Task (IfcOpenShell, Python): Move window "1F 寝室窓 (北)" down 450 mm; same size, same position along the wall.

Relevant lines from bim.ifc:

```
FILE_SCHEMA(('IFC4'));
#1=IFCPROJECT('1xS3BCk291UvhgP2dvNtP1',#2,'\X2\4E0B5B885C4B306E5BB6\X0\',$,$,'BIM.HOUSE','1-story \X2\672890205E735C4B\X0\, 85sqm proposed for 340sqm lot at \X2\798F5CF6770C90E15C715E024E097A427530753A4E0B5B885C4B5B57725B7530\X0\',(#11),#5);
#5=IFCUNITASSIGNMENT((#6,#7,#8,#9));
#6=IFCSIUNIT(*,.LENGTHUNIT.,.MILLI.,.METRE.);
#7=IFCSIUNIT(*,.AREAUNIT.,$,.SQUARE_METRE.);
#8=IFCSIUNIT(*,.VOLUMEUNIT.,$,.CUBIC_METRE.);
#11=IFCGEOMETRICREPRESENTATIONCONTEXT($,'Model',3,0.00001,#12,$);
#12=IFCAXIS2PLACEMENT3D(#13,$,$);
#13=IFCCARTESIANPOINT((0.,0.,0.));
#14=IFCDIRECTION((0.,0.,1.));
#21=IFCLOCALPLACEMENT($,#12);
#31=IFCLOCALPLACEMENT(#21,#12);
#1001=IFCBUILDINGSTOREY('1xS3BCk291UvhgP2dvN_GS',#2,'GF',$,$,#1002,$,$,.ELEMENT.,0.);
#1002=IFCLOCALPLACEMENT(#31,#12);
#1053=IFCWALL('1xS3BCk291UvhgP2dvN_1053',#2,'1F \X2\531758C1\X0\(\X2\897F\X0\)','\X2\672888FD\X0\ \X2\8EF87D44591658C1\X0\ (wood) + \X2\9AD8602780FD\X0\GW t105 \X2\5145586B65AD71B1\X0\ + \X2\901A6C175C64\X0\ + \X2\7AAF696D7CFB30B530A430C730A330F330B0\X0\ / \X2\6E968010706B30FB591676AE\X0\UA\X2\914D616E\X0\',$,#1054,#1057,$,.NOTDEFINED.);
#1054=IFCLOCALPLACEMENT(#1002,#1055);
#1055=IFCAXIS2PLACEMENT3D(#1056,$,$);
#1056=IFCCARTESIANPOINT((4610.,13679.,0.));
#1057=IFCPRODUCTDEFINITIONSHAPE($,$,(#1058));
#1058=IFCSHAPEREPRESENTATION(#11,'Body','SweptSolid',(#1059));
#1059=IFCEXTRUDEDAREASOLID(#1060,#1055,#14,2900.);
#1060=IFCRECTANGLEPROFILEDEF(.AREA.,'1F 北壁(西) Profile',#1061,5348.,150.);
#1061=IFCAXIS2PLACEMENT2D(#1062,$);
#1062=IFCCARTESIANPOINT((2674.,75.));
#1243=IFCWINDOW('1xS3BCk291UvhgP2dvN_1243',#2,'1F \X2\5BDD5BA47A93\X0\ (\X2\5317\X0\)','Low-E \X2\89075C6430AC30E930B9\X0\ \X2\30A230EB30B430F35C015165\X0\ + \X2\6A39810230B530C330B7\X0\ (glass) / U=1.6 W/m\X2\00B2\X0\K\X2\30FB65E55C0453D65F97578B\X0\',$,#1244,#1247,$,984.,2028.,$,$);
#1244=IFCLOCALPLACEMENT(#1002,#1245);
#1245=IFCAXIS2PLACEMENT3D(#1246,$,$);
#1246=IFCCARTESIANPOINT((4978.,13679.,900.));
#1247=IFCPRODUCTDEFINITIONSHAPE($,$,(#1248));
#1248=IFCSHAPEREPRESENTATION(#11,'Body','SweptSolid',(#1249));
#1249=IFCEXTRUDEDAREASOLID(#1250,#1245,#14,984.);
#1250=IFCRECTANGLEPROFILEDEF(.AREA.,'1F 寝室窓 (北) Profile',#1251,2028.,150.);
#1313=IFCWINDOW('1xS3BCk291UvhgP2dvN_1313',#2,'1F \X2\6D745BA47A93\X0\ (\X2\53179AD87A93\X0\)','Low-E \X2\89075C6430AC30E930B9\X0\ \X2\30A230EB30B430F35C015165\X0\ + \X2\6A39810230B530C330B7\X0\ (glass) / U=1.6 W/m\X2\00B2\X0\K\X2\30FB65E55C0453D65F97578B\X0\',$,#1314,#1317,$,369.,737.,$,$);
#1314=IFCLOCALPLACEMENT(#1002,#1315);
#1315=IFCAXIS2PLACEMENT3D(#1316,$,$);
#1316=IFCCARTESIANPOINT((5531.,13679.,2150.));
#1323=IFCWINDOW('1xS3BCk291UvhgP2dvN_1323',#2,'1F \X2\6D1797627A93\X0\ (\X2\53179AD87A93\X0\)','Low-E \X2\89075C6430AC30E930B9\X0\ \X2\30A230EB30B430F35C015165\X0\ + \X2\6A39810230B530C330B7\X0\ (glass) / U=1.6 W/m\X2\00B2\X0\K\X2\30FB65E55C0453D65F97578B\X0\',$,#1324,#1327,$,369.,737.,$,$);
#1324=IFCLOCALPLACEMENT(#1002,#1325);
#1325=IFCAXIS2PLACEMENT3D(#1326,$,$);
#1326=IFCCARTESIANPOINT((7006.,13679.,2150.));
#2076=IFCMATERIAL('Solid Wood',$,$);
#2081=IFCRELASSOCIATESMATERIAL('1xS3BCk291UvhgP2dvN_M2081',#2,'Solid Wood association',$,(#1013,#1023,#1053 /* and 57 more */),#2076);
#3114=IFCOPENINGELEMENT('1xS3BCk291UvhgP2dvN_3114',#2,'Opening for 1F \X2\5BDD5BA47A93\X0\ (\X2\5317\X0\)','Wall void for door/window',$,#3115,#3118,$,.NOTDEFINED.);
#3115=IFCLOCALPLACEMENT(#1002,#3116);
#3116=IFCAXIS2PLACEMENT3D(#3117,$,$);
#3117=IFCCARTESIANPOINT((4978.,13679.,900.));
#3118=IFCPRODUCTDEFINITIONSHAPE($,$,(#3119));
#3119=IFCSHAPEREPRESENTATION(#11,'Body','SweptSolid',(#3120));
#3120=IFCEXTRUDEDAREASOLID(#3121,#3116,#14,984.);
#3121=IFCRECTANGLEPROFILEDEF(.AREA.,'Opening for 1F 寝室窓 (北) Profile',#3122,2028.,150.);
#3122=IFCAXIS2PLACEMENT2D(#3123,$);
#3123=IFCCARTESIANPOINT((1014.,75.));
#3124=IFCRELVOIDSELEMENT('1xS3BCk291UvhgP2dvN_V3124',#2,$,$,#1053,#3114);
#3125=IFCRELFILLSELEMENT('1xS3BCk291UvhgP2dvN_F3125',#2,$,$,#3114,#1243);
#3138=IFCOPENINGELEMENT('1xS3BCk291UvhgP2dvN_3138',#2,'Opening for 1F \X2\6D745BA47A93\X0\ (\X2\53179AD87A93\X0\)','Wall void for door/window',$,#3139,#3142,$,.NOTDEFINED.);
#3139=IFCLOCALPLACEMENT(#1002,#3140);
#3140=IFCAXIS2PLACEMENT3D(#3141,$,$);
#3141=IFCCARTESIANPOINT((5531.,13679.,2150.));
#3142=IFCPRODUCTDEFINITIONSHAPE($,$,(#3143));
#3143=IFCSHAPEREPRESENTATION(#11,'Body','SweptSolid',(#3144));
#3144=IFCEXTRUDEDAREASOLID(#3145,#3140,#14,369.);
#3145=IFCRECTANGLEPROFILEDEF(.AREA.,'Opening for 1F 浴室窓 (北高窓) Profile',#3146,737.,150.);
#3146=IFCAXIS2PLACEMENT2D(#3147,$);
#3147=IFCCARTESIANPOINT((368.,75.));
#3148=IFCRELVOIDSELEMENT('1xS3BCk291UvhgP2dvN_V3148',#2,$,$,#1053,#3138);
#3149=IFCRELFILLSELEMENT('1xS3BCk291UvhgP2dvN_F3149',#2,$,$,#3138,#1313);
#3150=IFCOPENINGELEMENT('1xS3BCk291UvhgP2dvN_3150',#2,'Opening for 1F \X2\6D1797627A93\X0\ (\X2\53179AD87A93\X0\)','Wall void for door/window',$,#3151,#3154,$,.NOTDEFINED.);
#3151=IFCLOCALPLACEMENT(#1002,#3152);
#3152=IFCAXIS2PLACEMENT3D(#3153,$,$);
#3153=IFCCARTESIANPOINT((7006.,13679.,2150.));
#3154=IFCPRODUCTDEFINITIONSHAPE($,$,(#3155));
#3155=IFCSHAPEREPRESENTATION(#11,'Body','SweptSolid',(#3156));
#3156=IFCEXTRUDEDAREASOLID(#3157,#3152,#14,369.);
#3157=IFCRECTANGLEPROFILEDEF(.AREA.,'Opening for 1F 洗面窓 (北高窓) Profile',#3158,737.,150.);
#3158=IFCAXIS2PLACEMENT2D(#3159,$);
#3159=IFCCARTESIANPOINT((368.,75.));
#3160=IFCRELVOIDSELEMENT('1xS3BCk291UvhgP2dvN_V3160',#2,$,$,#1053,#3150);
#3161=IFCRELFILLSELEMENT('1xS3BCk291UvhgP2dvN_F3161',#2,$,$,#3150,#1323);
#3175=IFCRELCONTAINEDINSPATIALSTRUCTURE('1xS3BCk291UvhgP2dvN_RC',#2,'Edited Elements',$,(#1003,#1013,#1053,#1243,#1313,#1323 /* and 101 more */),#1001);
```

```python
import numpy as np
import ifcopenshell
import ifcopenshell.api.geometry
import ifcopenshell.util.placement
import ifcopenshell.util.unit

model = ifcopenshell.open("bim.ifc")
unit_scale = ifcopenshell.util.unit.calculate_unit_scale(model)

window = model.by_id(1243)
opening = window.FillsVoids[0].RelatingOpeningElement
dz = -450.0

shift = np.array([0.0, 0.0, dz])
# The window is not placed relative to its opening, so move both.
for product in (opening, window):
    matrix = ifcopenshell.util.placement.get_local_placement(product.ObjectPlacement)
    matrix[:3, 3] += shift
    ifcopenshell.api.geometry.edit_object_placement(model, product=product, matrix=matrix, is_si=False)

print(f"moved by {dz * unit_scale:+.3f} m")

model.write("bim_v2.ifc")
```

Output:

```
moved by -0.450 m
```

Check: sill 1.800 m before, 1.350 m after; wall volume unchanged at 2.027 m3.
